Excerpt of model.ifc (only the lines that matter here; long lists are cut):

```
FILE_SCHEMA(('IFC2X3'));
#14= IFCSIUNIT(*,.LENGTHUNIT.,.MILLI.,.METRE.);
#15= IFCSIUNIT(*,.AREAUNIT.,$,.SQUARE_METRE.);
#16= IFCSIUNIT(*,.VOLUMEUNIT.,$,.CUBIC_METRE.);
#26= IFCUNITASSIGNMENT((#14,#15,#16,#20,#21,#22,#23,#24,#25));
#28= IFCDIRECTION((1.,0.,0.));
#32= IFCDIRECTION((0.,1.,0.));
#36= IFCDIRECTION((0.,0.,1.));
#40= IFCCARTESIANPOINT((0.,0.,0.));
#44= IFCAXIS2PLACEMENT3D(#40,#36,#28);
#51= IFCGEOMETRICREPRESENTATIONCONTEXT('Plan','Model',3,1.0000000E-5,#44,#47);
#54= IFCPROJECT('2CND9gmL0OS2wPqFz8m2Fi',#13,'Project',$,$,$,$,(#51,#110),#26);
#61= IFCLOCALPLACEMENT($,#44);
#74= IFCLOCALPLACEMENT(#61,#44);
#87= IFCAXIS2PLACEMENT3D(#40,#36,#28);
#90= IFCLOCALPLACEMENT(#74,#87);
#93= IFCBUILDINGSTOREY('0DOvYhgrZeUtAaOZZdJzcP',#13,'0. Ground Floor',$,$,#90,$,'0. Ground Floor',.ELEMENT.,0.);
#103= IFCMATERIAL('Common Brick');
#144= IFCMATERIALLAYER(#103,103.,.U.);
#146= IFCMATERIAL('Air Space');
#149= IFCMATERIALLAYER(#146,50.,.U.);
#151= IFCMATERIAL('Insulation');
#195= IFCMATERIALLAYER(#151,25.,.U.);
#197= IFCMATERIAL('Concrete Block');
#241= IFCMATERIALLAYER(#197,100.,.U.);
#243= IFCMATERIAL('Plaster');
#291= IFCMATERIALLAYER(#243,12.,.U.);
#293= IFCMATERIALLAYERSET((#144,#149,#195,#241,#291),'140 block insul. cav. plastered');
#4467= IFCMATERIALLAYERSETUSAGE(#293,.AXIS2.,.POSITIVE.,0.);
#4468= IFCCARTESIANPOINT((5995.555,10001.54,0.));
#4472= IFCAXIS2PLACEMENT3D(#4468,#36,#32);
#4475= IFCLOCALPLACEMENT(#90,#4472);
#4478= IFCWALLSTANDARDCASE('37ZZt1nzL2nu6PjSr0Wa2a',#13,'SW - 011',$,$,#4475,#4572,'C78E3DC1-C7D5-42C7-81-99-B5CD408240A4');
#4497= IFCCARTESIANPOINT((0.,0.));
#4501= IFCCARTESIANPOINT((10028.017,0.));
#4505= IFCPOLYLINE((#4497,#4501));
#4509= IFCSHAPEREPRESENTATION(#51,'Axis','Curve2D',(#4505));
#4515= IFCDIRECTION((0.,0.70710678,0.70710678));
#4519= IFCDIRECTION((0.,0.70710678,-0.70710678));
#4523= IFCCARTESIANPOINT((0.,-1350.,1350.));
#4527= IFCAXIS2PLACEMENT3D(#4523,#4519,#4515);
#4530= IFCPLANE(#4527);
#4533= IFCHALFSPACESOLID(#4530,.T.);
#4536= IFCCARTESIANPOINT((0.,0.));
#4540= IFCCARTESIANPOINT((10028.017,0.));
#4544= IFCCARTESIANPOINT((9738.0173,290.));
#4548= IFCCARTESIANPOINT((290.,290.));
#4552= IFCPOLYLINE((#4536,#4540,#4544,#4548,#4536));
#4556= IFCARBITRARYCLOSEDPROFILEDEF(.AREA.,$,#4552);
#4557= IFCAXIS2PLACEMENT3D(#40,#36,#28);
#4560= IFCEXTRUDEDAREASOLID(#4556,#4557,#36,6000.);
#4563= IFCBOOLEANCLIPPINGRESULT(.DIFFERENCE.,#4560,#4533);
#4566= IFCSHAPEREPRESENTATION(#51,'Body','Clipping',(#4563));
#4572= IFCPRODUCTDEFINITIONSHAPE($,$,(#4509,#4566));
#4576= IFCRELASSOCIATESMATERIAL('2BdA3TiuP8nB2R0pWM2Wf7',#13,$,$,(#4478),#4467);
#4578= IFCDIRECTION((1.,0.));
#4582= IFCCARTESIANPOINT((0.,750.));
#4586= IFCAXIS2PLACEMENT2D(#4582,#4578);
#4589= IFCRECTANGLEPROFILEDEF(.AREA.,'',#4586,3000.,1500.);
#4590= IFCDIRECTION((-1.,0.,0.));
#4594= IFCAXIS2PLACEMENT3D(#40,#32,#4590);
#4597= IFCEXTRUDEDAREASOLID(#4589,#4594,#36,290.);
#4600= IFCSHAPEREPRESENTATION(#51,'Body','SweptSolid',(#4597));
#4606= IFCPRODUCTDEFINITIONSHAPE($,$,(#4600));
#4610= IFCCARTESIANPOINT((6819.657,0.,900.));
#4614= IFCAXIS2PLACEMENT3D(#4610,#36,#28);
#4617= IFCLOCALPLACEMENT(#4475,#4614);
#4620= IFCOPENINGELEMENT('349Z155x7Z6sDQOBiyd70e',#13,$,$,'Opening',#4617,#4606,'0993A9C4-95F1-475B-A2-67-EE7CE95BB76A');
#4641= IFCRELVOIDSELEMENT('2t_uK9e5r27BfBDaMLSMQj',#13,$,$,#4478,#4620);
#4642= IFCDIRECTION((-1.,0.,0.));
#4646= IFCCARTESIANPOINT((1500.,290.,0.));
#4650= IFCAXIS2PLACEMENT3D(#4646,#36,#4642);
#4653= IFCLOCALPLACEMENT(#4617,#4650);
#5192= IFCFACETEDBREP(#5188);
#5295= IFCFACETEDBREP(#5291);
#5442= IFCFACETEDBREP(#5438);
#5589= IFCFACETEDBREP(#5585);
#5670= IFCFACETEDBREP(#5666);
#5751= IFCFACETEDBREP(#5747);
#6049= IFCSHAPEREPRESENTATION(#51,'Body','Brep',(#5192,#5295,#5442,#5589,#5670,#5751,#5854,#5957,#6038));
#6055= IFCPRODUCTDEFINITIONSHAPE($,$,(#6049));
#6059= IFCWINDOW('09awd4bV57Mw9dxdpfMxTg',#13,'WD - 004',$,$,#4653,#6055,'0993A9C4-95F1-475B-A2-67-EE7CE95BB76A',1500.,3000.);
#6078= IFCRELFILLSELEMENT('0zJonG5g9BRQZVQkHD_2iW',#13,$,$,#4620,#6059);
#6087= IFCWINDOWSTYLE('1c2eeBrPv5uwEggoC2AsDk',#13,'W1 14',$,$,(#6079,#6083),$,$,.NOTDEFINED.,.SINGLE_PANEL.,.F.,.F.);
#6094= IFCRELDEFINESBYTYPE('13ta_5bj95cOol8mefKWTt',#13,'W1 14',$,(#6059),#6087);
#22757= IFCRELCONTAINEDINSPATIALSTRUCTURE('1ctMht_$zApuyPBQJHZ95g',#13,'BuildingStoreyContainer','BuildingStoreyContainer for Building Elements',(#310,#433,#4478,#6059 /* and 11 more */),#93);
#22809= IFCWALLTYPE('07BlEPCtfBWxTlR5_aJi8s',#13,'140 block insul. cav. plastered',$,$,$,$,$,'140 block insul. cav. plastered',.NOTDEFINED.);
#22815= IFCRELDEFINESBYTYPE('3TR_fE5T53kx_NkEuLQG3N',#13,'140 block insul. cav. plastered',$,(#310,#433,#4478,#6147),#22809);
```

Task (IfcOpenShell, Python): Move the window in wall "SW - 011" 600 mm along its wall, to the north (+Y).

```python
import ifcopenshell
import ifcopenshell.api.geometry
import ifcopenshell.util.placement
import ifcopenshell.util.unit

model = ifcopenshell.open("model.ifc")
unit_scale = ifcopenshell.util.unit.calculate_unit_scale(model)

window = model.by_guid("09awd4bV57Mw9dxdpfMxTg")
opening = window.FillsVoids[0].RelatingOpeningElement
wall = opening.VoidsElements[0].RelatingBuildingElement

wall_matrix = ifcopenshell.util.placement.get_local_placement(wall.ObjectPlacement)
shift = wall_matrix[:3, 0] * 0.6 / unit_scale
before = ifcopenshell.util.placement.get_local_placement(window.ObjectPlacement)[:3, 3].copy()

# The window is placed relative to its opening, so it follows when the opening moves.
matrix = ifcopenshell.util.placement.get_local_placement(opening.ObjectPlacement)
matrix[:3, 3] += shift
ifcopenshell.api.geometry.edit_object_placement(
    model, product=opening, matrix=matrix, is_si=False, should_transform_children=True
)

after = ifcopenshell.util.placement.get_local_placement(window.ObjectPlacement)[:3, 3]
print("window moved by", (after - before).round(3) + 0.0)

model.write("model_v2.ifc")
```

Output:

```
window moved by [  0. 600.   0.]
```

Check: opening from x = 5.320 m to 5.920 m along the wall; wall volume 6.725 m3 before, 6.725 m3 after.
